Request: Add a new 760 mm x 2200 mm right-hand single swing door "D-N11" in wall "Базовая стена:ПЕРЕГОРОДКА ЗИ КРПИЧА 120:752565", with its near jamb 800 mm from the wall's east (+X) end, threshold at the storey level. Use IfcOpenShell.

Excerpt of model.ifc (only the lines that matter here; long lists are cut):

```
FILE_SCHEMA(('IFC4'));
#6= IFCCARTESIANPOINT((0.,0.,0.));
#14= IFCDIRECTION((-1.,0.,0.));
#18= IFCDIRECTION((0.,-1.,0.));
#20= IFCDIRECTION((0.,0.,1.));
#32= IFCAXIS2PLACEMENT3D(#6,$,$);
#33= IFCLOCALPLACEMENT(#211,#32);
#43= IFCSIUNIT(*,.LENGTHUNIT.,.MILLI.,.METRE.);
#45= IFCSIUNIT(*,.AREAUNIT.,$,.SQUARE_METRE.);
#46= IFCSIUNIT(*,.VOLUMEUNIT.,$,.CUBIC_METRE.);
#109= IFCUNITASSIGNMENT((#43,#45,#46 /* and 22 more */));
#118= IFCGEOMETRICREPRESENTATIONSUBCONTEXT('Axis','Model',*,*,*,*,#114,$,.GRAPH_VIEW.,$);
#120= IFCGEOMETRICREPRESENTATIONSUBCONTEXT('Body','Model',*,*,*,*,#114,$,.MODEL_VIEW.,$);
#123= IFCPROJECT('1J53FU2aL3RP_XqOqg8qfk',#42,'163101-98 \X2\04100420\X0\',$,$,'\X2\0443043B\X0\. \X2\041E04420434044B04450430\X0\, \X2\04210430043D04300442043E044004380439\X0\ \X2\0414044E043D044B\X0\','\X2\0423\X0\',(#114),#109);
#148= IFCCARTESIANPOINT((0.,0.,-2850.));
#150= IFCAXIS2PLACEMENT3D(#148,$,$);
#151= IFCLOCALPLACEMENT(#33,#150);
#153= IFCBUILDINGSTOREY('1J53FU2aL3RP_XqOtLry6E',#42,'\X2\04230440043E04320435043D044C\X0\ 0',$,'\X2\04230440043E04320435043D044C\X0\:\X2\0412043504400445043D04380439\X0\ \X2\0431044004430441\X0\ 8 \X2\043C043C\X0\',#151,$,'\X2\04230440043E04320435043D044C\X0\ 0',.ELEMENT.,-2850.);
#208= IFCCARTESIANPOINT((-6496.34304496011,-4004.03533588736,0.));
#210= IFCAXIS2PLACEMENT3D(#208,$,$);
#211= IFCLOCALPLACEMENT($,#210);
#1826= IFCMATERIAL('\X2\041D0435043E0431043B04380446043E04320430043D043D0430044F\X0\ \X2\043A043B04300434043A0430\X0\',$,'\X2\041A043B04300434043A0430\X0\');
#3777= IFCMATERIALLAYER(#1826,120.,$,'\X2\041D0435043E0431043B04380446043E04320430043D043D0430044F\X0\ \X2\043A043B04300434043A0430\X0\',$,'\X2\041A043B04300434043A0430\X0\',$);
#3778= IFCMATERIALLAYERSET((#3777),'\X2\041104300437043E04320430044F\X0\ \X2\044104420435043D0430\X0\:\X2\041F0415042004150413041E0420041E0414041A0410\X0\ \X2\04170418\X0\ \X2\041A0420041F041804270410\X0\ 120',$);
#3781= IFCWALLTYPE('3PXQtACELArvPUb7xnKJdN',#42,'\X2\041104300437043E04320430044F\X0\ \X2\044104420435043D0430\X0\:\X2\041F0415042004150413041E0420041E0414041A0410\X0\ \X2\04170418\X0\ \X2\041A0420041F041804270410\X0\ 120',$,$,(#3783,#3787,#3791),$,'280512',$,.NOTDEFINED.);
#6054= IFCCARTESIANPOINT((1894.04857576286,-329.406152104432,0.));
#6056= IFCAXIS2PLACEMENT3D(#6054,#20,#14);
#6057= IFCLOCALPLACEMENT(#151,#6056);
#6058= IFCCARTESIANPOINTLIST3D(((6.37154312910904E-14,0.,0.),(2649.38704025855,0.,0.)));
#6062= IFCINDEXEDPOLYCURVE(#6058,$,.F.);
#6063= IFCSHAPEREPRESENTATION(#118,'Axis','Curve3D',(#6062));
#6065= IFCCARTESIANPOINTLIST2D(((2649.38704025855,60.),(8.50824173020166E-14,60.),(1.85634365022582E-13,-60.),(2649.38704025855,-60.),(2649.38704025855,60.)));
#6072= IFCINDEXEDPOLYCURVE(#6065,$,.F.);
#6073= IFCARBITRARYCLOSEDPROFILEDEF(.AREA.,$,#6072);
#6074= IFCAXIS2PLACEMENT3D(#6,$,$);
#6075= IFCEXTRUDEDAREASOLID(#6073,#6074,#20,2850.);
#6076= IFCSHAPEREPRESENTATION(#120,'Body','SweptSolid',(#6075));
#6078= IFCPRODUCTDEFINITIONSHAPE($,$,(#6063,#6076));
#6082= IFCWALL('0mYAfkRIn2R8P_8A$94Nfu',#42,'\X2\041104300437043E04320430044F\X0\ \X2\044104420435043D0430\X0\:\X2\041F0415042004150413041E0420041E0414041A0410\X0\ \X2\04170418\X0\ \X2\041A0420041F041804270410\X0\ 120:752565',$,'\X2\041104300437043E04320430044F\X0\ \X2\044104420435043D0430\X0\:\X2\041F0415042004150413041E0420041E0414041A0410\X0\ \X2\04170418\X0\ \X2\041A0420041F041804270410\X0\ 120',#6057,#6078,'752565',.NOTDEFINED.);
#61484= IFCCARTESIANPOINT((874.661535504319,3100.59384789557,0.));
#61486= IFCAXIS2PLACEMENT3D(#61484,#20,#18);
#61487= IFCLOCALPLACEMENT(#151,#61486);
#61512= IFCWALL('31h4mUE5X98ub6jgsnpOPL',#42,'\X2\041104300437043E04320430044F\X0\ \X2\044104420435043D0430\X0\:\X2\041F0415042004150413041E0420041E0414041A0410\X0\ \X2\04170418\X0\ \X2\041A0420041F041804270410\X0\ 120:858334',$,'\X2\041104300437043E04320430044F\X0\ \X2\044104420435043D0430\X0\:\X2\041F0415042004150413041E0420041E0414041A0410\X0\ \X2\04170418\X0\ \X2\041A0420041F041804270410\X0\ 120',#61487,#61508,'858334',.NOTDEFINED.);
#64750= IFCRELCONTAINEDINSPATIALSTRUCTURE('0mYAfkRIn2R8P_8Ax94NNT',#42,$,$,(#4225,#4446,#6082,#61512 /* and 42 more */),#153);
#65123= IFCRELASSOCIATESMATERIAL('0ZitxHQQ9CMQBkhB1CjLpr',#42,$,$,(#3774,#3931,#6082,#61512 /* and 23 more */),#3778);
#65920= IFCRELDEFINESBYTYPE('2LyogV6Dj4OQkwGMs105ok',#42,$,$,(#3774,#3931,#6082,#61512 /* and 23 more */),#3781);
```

```python
import numpy as np
import ifcopenshell
import ifcopenshell.api.feature
import ifcopenshell.api.geometry
import ifcopenshell.api.root
import ifcopenshell.api.spatial
import ifcopenshell.geom
import ifcopenshell.util.element
import ifcopenshell.util.placement
import ifcopenshell.util.representation
import ifcopenshell.util.shape
import ifcopenshell.util.unit

model = ifcopenshell.open("model.ifc")
unit_scale = ifcopenshell.util.unit.calculate_unit_scale(model)
settings = ifcopenshell.geom.settings()


def volume(element):
    """Net volume in cubic metres, openings subtracted."""
    shape = ifcopenshell.geom.create_shape(settings, element)
    return ifcopenshell.util.shape.get_volume(shape.geometry)


wall = model.by_id(6082)
storey = ifcopenshell.util.element.get_container(wall, ifc_class="IfcBuildingStorey")
context = ifcopenshell.util.representation.get_context(model, "Model", "Body", "MODEL_VIEW")
before = volume(wall)

width, height, from_end, sill = 0.76, 2.2, 0.8, 0.0  # metres

# The wall runs along its own X axis, and the end named is its -X end.
wall_shape = ifcopenshell.geom.create_shape(settings, wall)
x, y, z = ifcopenshell.util.shape.get_vertices(wall_shape.geometry).T
start = x.min() + from_end
face, thickness = float(y.min()), float(y.max() - y.min())
wall_matrix = ifcopenshell.util.placement.get_local_placement(wall.ObjectPlacement)
level = ifcopenshell.util.placement.get_local_placement(storey.ObjectPlacement)[2, 3]


def in_wall(x, y):
    """Placement at x, y metres in the wall's axes, at sill height."""
    matrix = wall_matrix.copy()
    matrix[:, 3] = wall_matrix @ np.array([x / unit_scale, y / unit_scale, 0.0, 1.0])
    matrix[2, 3] = level + sill / unit_scale
    return matrix


# Opening: a box that overshoots both wall faces by 50 mm.
opening = ifcopenshell.api.root.create_entity(model, ifc_class="IfcOpeningElement", predefined_type="OPENING")
box = ifcopenshell.api.geometry.add_wall_representation(
    model, context=context, length=width, height=height, thickness=thickness + 0.1
)
ifcopenshell.api.geometry.assign_representation(model, product=opening, representation=box)
ifcopenshell.api.geometry.edit_object_placement(model, product=opening, matrix=in_wall(start, face - 0.05), is_si=False)
ifcopenshell.api.feature.add_feature(model, feature=opening, element=wall)

door = ifcopenshell.api.root.create_entity(model, ifc_class="IfcDoor", name="D-N11", predefined_type="DOOR")
door.OverallWidth, door.OverallHeight = width / unit_scale, height / unit_scale
door.OperationType = "SINGLE_SWING_RIGHT"
body = ifcopenshell.api.geometry.add_door_representation(
    model,
    context=context,
    overall_width=door.OverallWidth,
    overall_height=door.OverallHeight,
    operation_type="SINGLE_SWING_RIGHT",
    lining_properties={"LiningDepth": thickness / unit_scale, "ThresholdDepth": thickness / unit_scale},
)
ifcopenshell.api.geometry.assign_representation(model, product=door, representation=body)
ifcopenshell.api.spatial.assign_container(model, products=[door], relating_structure=storey)
ifcopenshell.api.feature.add_filling(model, opening=opening, element=door)

# The lining spans the wall, so the door starts at the wall face.
ifcopenshell.api.geometry.edit_object_placement(model, product=door, matrix=in_wall(start, face), is_si=False)

after = volume(wall)

print(f"wall volume {before:.3f} -> {after:.3f} m3")

model.write("model_updated.ifc")
```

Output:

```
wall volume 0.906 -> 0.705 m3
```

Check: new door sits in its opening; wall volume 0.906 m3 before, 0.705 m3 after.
